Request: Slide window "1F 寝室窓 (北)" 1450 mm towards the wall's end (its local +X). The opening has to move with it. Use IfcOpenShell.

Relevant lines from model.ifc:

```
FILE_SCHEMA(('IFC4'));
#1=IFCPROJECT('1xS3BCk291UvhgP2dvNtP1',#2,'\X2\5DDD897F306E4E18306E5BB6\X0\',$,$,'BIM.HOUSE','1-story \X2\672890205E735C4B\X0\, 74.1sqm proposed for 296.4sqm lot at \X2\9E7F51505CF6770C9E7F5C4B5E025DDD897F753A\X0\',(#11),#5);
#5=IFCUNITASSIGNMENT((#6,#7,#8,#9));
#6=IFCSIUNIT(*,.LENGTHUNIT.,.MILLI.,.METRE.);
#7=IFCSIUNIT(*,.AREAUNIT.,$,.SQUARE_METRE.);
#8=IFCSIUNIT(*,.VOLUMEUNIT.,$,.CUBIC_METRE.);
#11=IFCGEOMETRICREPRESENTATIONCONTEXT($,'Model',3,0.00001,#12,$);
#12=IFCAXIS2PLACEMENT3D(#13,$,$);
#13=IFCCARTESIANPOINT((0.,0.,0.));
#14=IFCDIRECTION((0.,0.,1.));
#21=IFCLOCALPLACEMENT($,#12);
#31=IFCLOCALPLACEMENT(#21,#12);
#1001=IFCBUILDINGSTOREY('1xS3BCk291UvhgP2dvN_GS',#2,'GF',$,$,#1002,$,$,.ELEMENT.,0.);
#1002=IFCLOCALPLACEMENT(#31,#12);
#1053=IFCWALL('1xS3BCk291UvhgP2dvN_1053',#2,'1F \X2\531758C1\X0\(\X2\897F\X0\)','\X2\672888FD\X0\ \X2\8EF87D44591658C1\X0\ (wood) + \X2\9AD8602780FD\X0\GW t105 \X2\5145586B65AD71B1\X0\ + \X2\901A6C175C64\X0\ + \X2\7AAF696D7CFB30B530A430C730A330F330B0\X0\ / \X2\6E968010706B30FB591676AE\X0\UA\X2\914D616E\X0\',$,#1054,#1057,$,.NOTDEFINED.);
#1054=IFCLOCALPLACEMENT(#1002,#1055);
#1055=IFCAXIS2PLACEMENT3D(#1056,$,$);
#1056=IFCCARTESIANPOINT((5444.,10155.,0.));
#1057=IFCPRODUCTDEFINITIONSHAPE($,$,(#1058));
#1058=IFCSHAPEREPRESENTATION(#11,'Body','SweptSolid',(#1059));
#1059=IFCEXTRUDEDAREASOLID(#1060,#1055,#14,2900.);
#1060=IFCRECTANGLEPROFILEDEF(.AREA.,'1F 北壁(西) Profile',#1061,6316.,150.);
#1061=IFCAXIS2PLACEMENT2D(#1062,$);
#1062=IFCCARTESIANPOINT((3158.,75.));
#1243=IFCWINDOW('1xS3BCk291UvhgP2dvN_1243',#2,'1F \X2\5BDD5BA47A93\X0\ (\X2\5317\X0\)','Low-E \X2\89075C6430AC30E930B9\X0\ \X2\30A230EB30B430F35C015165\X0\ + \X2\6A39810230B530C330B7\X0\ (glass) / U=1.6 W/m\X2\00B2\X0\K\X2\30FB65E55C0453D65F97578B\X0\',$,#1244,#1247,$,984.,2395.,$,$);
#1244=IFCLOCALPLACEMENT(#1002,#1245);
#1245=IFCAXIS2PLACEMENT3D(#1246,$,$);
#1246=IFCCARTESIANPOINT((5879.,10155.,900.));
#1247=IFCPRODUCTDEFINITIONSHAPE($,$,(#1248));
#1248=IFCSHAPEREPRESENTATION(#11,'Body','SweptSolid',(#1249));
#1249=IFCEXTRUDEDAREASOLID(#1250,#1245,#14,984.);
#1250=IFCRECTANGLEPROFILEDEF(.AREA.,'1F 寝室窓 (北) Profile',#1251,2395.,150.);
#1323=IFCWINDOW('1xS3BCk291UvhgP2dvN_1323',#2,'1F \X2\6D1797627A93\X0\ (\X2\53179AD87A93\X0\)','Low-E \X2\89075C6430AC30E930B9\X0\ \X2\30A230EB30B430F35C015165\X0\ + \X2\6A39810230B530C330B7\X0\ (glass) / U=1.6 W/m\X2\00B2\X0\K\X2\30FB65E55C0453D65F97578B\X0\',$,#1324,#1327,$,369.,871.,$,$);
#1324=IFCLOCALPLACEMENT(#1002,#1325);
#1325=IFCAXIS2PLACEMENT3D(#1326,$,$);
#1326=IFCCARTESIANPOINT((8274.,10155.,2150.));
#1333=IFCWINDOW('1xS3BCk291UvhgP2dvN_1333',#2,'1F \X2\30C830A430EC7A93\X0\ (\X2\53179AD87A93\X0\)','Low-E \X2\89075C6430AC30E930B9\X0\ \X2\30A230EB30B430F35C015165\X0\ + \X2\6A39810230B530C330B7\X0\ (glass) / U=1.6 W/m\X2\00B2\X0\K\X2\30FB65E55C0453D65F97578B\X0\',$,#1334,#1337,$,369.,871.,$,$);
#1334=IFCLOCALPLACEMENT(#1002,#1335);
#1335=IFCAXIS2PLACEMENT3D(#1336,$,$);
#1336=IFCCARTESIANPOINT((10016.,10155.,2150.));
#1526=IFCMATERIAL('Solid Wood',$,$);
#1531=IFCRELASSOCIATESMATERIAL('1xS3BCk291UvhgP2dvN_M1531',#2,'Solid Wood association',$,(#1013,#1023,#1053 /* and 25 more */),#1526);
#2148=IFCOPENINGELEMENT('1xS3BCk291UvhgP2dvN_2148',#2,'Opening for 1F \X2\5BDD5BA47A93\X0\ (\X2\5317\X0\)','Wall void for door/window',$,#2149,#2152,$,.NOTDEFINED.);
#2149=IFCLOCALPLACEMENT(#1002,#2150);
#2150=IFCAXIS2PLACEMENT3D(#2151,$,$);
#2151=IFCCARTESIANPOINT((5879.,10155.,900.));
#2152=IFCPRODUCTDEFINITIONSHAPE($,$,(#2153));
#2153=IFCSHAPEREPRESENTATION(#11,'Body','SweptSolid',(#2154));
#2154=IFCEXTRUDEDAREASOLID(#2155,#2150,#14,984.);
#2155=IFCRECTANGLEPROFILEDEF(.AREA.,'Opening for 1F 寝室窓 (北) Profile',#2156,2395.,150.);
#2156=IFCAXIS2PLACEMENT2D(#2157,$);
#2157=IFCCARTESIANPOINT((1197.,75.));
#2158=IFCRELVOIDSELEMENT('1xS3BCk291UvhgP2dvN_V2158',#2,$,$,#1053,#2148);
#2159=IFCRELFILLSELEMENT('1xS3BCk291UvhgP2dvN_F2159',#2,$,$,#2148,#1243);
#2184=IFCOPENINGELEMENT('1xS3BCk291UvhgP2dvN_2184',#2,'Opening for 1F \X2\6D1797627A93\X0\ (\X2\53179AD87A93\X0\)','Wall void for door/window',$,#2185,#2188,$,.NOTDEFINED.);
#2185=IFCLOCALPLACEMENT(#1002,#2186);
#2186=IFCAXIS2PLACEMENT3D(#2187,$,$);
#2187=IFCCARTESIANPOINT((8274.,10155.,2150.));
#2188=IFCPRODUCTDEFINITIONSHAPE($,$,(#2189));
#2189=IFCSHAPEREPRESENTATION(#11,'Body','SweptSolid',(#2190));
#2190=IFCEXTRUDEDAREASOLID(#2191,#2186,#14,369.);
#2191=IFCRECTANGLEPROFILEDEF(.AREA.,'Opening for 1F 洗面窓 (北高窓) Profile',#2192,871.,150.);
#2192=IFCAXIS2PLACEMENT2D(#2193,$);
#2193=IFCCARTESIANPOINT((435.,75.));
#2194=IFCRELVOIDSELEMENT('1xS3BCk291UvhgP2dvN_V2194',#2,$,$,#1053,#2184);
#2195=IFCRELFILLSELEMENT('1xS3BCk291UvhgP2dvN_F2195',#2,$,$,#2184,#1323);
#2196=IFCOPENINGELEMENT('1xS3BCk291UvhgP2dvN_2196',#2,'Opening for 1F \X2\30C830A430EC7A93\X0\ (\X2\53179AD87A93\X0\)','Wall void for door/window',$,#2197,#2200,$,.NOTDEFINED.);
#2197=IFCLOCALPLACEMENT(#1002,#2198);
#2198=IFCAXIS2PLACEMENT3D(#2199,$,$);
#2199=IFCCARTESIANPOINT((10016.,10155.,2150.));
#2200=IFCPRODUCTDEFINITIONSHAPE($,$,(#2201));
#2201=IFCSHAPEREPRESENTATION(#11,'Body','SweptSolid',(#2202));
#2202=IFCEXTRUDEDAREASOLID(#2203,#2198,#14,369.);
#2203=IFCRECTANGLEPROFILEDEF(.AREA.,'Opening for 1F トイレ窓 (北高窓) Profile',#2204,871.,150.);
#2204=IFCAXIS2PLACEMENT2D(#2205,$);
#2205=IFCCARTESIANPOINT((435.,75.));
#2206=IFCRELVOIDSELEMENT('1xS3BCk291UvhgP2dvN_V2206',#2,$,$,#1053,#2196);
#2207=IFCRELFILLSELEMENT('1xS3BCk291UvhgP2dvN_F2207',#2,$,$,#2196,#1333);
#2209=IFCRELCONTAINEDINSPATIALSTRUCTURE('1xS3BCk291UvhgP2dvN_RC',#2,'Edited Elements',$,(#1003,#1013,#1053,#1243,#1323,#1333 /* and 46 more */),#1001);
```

```python
import ifcopenshell
import ifcopenshell.api.geometry
import ifcopenshell.util.placement
import ifcopenshell.util.unit

model = ifcopenshell.open("model.ifc")
unit_scale = ifcopenshell.util.unit.calculate_unit_scale(model)

window = model.by_guid("1xS3BCk291UvhgP2dvN_1243")
opening = window.FillsVoids[0].RelatingOpeningElement
wall = opening.VoidsElements[0].RelatingBuildingElement

wall_matrix = ifcopenshell.util.placement.get_local_placement(wall.ObjectPlacement)
shift = wall_matrix[:3, 0] * 1.45 / unit_scale
before = ifcopenshell.util.placement.get_local_placement(window.ObjectPlacement)[:3, 3].copy()

# The window is not placed relative to its opening, so move both.
for product in (opening, window):
    matrix = ifcopenshell.util.placement.get_local_placement(product.ObjectPlacement)
    matrix[:3, 3] += shift
    ifcopenshell.api.geometry.edit_object_placement(model, product=product, matrix=matrix, is_si=False)

after = ifcopenshell.util.placement.get_local_placement(window.ObjectPlacement)[:3, 3]
print("window moved by", (after - before).round(3) + 0.0)

model.write("model_updated.ifc")
```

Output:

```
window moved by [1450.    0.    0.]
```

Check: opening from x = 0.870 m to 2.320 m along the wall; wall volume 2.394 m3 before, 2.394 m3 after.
